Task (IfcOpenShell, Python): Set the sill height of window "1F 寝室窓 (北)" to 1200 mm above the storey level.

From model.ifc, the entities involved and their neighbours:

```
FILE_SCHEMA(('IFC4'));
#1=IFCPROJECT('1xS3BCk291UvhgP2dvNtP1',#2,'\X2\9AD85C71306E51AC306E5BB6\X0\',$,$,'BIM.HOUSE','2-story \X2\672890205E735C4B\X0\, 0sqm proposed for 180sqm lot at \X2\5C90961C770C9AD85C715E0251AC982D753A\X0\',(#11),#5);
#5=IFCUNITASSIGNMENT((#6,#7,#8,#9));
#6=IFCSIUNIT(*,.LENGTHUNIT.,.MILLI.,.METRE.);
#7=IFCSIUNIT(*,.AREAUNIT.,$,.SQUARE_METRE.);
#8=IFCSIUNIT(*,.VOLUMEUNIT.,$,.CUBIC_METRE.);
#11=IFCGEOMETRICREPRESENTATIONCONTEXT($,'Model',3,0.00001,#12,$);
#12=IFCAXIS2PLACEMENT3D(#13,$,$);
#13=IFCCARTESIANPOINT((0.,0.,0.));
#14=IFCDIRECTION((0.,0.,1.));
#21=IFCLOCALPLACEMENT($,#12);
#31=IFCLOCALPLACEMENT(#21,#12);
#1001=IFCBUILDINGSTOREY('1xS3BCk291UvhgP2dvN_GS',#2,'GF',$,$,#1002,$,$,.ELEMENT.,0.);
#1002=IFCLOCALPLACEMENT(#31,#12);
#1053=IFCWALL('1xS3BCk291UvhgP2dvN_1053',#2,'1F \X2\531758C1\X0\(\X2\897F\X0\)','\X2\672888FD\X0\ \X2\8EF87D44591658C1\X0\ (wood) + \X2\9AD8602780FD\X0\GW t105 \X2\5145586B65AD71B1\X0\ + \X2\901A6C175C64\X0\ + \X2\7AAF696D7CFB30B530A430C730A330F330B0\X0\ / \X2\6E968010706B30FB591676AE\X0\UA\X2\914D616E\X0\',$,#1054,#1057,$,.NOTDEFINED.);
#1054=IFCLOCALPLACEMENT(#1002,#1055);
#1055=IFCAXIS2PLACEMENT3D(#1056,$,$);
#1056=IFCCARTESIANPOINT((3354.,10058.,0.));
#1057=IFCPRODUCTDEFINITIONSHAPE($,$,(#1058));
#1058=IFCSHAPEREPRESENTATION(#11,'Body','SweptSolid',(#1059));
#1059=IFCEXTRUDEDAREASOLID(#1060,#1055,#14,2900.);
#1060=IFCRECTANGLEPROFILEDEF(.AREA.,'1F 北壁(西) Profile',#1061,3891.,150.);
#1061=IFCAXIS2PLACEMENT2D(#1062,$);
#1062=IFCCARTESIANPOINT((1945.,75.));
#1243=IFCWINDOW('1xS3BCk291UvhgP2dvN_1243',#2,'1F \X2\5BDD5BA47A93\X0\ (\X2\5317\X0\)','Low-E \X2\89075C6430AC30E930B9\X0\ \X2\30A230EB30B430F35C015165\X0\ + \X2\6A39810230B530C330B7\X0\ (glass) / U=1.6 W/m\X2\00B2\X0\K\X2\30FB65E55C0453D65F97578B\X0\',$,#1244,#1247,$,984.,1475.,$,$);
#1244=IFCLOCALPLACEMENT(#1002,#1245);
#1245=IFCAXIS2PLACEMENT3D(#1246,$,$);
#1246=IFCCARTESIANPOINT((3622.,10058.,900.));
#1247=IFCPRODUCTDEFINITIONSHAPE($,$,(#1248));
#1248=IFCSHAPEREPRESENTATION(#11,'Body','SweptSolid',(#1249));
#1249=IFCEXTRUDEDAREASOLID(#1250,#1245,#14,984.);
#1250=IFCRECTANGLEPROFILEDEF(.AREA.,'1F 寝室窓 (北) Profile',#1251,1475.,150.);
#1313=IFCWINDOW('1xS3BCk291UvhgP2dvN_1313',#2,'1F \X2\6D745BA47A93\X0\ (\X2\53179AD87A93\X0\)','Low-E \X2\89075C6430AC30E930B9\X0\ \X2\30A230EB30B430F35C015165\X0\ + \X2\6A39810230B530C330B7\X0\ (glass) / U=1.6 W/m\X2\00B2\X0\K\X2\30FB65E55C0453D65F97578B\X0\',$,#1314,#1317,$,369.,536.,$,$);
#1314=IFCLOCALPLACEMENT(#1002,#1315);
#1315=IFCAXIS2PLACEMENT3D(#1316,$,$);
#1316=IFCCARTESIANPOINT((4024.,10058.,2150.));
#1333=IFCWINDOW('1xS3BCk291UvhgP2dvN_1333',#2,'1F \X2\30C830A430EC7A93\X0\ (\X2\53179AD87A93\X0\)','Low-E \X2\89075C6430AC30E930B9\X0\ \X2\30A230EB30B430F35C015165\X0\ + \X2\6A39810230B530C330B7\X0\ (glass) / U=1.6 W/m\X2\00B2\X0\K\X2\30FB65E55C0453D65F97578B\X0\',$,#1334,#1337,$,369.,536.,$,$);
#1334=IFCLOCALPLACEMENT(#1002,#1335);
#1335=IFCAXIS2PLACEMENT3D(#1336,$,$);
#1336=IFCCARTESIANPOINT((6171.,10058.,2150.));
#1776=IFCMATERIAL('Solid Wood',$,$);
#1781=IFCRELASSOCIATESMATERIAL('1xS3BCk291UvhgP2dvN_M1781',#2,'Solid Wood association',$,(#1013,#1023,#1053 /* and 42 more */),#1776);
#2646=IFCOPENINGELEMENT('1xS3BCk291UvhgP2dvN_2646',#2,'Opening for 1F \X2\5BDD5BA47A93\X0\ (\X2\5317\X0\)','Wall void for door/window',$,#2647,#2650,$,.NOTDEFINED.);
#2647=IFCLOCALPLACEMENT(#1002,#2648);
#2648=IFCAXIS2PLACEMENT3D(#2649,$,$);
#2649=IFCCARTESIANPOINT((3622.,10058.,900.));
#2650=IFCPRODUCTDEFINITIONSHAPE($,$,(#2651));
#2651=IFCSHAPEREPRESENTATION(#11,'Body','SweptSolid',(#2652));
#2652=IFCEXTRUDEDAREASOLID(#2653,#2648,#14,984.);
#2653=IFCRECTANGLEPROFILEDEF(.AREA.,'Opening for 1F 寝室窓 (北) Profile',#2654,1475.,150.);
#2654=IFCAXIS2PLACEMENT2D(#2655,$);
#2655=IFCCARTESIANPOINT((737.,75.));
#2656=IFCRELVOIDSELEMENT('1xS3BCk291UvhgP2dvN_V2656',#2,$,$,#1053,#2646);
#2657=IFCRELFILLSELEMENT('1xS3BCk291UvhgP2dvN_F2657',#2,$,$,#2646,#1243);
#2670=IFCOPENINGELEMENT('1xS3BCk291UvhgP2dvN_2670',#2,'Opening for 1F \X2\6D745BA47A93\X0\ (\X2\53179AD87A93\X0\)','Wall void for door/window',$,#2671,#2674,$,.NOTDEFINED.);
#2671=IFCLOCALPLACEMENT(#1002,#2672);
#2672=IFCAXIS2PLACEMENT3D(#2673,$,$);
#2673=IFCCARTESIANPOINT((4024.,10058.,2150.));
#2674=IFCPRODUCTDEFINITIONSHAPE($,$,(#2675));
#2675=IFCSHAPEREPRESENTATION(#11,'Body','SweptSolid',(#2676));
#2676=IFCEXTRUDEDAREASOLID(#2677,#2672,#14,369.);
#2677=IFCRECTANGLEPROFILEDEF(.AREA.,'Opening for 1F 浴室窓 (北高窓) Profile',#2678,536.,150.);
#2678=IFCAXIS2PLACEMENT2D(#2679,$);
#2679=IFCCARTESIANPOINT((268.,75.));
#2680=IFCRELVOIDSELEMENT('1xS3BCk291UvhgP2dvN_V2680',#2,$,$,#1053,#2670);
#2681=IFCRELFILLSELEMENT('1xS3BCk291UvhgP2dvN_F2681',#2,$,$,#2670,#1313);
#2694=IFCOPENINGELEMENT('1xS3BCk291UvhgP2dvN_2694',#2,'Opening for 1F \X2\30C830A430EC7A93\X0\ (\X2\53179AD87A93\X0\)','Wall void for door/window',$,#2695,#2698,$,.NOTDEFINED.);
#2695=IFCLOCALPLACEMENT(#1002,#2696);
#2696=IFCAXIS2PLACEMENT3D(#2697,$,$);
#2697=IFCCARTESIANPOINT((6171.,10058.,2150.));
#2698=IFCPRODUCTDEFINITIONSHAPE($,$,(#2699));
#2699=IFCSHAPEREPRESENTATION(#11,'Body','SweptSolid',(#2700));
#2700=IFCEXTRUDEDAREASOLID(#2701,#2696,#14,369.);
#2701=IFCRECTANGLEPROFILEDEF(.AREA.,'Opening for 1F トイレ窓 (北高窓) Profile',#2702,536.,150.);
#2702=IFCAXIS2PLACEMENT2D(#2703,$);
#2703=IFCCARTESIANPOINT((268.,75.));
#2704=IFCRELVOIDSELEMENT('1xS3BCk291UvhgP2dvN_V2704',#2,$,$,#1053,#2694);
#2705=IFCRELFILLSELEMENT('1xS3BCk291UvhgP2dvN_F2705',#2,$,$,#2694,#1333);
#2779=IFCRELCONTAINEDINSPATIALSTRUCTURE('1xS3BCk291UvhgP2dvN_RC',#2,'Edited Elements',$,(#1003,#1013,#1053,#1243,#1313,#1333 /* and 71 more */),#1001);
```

```python
import numpy as np
import ifcopenshell
import ifcopenshell.api.geometry
import ifcopenshell.geom
import ifcopenshell.util.element
import ifcopenshell.util.placement
import ifcopenshell.util.shape
import ifcopenshell.util.unit

model = ifcopenshell.open("model.ifc")
unit_scale = ifcopenshell.util.unit.calculate_unit_scale(model)

window = model.by_id(1243)
opening = window.FillsVoids[0].RelatingOpeningElement
storey = ifcopenshell.util.element.get_container(window, ifc_class="IfcBuildingStorey")
level = ifcopenshell.util.placement.get_local_placement(storey.ObjectPlacement)[2, 3]

# The opening's origin need not be at the sill, so measure its lowest point.
shape = ifcopenshell.geom.create_shape(ifcopenshell.geom.settings(), opening)
bottom = ifcopenshell.util.shape.get_shape_bottom_elevation(shape, shape.geometry) / unit_scale
dz = level + 1200.0 - bottom

shift = np.array([0.0, 0.0, dz])
# The window is not placed relative to its opening, so move both.
for product in (opening, window):
    matrix = ifcopenshell.util.placement.get_local_placement(product.ObjectPlacement)
    matrix[:3, 3] += shift
    ifcopenshell.api.geometry.edit_object_placement(model, product=product, matrix=matrix, is_si=False)

print(f"moved by {dz * unit_scale:+.3f} m")

model.write("model_edited.ifc")
```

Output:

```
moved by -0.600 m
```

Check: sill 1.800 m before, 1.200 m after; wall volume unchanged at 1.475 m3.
